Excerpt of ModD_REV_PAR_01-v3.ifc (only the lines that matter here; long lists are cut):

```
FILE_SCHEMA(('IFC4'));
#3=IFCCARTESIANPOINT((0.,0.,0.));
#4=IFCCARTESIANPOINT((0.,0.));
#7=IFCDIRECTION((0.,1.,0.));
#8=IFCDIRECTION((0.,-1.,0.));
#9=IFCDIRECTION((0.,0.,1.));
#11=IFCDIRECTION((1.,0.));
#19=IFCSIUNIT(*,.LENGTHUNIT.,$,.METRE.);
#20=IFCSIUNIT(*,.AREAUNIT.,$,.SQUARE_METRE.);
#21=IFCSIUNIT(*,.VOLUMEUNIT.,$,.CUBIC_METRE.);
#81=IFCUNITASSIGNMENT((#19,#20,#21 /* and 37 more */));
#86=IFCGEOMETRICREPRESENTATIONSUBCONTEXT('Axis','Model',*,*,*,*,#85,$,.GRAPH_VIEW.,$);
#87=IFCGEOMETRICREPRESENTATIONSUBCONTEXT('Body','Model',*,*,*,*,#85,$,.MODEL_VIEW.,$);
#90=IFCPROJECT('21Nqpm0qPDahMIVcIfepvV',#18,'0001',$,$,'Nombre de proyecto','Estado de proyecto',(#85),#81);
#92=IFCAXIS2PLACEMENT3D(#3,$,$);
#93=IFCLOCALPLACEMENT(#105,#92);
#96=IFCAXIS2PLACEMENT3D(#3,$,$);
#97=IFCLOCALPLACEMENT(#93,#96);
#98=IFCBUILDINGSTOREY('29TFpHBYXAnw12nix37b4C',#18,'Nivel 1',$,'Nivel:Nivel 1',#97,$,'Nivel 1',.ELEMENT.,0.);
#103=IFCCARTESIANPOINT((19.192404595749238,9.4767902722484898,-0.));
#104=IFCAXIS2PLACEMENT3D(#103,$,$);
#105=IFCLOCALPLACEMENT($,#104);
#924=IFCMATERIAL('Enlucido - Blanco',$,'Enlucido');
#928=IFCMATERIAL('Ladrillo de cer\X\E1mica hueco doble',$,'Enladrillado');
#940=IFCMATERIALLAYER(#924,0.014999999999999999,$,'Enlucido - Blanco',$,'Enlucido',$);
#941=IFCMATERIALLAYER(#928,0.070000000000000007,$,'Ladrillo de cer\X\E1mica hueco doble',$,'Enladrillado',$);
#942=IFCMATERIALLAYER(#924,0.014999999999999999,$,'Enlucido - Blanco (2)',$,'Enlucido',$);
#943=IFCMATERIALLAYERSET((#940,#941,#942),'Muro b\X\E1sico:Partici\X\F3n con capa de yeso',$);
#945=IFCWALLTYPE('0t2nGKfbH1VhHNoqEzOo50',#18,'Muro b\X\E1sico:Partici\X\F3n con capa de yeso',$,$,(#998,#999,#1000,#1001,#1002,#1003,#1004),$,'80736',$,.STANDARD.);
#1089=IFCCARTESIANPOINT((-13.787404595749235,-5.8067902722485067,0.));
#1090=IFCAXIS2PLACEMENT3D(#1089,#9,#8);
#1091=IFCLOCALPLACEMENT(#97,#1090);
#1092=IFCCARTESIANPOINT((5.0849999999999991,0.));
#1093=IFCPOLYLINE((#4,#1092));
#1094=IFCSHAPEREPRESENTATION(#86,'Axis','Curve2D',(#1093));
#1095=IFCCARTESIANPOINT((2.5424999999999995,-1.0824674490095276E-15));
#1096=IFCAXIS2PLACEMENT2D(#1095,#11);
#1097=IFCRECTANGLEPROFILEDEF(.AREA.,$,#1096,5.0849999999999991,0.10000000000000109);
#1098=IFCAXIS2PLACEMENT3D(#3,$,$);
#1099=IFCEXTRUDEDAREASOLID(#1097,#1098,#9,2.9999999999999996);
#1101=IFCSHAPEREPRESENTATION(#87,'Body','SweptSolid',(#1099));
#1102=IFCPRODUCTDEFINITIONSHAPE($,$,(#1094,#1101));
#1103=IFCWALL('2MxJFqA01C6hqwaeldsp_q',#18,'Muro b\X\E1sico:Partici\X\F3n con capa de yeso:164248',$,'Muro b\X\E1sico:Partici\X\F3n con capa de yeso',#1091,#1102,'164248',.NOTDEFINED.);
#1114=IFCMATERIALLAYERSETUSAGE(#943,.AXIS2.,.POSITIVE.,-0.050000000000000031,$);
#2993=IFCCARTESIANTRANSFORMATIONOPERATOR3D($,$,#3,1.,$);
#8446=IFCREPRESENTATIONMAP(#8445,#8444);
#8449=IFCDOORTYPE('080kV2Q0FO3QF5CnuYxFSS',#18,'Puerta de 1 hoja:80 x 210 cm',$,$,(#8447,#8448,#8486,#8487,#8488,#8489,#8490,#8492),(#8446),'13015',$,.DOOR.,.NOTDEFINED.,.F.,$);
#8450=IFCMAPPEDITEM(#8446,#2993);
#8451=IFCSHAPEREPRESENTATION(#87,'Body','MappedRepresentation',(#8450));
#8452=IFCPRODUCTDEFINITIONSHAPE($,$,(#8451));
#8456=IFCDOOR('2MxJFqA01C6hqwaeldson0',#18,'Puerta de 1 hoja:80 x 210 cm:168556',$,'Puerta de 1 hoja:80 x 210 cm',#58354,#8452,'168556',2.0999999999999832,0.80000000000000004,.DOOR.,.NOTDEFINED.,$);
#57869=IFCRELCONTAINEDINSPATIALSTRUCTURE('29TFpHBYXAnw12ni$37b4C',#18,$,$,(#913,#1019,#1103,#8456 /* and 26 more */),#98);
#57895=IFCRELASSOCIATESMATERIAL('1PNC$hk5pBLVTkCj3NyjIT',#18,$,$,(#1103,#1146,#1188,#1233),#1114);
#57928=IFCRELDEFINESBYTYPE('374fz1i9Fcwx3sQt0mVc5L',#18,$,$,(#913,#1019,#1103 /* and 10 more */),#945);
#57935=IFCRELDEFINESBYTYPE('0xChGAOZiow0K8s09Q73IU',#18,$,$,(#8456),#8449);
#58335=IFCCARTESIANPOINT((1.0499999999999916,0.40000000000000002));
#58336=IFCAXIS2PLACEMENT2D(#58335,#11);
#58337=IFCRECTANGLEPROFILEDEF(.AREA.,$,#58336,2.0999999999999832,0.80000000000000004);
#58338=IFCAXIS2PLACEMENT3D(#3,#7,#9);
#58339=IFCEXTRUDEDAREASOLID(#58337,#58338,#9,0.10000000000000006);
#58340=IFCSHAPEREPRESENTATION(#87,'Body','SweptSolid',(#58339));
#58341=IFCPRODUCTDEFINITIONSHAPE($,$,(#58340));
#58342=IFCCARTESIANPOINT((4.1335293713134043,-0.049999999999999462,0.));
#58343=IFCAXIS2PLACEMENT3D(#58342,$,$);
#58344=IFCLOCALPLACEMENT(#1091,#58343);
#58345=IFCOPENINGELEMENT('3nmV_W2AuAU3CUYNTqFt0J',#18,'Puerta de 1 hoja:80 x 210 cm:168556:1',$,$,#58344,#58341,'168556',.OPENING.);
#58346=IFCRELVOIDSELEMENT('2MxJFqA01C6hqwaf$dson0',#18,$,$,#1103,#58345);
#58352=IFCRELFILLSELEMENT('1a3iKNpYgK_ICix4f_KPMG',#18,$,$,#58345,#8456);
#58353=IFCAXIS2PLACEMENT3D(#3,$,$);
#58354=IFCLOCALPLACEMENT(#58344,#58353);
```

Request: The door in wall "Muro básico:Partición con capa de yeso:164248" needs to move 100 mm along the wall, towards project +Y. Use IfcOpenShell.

```python
import ifcopenshell
import ifcopenshell.api.geometry
import ifcopenshell.util.placement
import ifcopenshell.util.unit

model = ifcopenshell.open("ModD_REV_PAR_01-v3.ifc")
unit_scale = ifcopenshell.util.unit.calculate_unit_scale(model)

door = model.by_guid("2MxJFqA01C6hqwaeldson0")
opening = door.FillsVoids[0].RelatingOpeningElement
wall = opening.VoidsElements[0].RelatingBuildingElement

wall_matrix = ifcopenshell.util.placement.get_local_placement(wall.ObjectPlacement)
shift = wall_matrix[:3, 0] * -0.1 / unit_scale
before = ifcopenshell.util.placement.get_local_placement(door.ObjectPlacement)[:3, 3].copy()

# The door is placed relative to its opening, so it follows when the opening moves.
matrix = ifcopenshell.util.placement.get_local_placement(opening.ObjectPlacement)
matrix[:3, 3] += shift
ifcopenshell.api.geometry.edit_object_placement(
    model, product=opening, matrix=matrix, is_si=False, should_transform_children=True
)

after = ifcopenshell.util.placement.get_local_placement(door.ObjectPlacement)[:3, 3]
print("door moved by", (after - before).round(3) + 0.0)

model.write("ModD_REV_PAR_01-v3_rev.ifc")
```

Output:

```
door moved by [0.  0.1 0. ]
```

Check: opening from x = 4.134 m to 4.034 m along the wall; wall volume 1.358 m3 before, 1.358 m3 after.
